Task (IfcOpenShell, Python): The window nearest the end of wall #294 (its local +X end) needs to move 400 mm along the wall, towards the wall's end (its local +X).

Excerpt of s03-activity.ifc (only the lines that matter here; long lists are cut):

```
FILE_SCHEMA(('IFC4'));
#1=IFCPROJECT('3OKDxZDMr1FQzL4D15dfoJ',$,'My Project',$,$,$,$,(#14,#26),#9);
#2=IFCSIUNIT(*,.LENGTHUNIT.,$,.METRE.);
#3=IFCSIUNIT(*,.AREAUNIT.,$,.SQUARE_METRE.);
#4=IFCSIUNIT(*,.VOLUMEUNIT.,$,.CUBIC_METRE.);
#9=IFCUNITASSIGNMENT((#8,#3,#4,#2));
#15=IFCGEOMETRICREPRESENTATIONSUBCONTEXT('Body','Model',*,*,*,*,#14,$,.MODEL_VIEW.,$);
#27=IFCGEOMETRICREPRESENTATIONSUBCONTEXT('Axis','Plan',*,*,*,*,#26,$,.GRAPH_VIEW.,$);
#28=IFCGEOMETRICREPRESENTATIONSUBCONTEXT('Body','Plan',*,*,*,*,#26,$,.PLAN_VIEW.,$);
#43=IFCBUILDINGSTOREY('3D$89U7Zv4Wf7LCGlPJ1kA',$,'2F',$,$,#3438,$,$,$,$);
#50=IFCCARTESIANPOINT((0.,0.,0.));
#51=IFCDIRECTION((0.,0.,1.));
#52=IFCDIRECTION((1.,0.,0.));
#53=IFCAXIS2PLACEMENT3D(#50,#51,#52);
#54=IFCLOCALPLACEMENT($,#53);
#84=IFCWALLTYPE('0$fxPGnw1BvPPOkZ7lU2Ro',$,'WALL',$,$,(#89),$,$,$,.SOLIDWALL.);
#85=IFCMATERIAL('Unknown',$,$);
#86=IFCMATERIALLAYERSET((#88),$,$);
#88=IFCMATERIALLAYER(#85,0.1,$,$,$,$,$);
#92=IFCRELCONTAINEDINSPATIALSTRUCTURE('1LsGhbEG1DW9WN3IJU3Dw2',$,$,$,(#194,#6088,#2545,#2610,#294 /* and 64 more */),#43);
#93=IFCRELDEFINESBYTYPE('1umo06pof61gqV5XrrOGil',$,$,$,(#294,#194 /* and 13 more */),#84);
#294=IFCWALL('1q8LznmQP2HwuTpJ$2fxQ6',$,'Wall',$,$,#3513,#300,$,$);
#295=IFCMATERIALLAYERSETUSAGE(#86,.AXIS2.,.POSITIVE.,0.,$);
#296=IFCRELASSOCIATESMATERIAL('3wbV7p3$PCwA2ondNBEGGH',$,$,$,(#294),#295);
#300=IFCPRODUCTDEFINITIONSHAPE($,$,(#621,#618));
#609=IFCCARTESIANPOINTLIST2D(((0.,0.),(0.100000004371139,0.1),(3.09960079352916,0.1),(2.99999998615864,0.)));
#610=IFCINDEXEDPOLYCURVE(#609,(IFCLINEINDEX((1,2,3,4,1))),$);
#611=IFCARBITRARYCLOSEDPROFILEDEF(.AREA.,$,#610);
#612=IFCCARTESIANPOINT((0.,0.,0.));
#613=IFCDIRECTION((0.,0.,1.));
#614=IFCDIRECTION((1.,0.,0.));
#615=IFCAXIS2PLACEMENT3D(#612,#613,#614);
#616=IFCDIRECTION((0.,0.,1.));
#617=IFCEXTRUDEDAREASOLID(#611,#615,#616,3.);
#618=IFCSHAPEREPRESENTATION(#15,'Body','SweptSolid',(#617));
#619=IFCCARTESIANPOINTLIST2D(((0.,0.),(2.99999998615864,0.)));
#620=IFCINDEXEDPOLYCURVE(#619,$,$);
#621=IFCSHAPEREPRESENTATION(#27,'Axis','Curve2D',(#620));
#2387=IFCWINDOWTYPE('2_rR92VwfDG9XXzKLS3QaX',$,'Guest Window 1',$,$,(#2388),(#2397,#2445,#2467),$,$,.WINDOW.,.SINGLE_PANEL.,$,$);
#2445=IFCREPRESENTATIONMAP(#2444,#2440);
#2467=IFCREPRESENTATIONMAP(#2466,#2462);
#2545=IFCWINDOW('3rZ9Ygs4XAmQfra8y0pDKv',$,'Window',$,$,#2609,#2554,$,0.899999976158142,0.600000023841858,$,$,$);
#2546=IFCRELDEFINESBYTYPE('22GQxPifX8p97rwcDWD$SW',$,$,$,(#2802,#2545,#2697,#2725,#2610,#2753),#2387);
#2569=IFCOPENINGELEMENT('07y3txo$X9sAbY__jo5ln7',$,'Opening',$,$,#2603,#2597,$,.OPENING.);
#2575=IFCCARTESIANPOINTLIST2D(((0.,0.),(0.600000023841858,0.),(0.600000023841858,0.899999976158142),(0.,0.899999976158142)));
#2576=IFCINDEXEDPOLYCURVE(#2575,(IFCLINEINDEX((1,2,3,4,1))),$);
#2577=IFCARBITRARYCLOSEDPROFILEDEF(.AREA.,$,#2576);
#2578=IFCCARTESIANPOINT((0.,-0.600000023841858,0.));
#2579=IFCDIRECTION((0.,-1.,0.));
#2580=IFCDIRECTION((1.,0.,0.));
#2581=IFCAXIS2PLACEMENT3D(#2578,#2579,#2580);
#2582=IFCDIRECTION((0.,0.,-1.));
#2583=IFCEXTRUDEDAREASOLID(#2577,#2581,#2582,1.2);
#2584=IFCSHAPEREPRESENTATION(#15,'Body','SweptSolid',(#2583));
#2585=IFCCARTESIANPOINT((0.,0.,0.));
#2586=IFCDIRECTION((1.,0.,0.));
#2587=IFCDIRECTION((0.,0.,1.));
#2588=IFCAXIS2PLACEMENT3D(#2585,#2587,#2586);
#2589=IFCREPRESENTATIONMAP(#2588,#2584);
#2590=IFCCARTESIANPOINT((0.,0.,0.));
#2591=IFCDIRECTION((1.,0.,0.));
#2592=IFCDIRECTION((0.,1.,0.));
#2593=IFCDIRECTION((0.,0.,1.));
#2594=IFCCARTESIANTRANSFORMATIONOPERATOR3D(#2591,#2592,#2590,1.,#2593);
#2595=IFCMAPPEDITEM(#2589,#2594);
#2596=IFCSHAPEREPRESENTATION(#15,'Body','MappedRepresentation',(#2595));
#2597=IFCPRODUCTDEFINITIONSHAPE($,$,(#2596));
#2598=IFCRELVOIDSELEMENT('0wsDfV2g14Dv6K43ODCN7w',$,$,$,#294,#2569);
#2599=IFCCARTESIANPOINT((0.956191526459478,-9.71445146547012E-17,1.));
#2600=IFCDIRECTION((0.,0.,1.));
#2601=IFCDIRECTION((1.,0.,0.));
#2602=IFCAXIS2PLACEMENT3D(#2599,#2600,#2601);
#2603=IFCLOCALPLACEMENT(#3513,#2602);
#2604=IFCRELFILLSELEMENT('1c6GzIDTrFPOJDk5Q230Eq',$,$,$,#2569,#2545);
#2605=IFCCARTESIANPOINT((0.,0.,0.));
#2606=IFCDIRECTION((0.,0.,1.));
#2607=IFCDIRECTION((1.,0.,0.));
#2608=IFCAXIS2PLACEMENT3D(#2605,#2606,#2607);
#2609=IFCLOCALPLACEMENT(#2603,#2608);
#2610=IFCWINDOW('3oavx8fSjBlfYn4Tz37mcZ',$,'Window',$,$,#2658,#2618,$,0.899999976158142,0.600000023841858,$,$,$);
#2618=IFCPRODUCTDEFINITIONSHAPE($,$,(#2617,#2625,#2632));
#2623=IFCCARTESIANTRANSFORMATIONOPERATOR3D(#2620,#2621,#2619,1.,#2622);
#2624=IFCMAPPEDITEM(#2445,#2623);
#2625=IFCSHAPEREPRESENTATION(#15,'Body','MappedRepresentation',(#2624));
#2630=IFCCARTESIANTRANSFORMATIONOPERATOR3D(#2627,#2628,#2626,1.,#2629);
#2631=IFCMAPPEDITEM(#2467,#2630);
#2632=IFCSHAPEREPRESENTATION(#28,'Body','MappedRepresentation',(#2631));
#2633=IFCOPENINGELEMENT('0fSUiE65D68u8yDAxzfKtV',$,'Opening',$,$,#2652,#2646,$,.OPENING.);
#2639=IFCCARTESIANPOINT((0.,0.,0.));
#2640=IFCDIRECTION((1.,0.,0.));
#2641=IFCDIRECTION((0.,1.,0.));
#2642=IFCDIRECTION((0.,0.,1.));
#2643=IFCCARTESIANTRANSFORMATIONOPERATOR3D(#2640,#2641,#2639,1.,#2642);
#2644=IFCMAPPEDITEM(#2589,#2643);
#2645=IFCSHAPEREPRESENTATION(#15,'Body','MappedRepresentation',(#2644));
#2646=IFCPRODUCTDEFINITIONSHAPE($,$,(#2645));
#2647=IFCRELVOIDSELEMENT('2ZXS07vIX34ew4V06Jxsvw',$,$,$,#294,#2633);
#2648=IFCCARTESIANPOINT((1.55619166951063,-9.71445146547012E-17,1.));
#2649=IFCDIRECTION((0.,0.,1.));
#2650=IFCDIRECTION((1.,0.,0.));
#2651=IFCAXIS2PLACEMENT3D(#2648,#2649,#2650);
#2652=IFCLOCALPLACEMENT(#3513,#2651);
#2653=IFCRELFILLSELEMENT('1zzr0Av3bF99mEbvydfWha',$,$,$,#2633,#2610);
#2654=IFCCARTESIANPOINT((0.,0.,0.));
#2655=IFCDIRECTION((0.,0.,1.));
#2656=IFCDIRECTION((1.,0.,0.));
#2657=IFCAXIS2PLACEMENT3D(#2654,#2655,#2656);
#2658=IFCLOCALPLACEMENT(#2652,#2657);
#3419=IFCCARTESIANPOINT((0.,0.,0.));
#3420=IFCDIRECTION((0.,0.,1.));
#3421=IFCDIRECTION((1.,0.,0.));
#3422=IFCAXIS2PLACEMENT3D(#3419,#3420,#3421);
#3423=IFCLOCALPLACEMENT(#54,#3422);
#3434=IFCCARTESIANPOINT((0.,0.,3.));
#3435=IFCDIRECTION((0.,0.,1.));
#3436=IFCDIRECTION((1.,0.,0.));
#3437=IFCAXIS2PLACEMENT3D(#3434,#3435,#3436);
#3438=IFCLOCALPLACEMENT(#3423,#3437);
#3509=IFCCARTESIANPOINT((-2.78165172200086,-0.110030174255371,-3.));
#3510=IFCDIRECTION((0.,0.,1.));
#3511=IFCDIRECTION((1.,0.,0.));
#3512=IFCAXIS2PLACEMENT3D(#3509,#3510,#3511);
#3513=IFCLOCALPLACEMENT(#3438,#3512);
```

```python
import ifcopenshell
import ifcopenshell.api.geometry
import ifcopenshell.util.placement
import ifcopenshell.util.unit

model = ifcopenshell.open("s03-activity.ifc")
unit_scale = ifcopenshell.util.unit.calculate_unit_scale(model)

window = model.by_guid("3oavx8fSjBlfYn4Tz37mcZ")
opening = window.FillsVoids[0].RelatingOpeningElement
wall = opening.VoidsElements[0].RelatingBuildingElement

wall_matrix = ifcopenshell.util.placement.get_local_placement(wall.ObjectPlacement)
shift = wall_matrix[:3, 0] * 0.4 / unit_scale
before = ifcopenshell.util.placement.get_local_placement(window.ObjectPlacement)[:3, 3].copy()

# The window is placed relative to its opening, so it follows when the opening moves.
matrix = ifcopenshell.util.placement.get_local_placement(opening.ObjectPlacement)
matrix[:3, 3] += shift
ifcopenshell.api.geometry.edit_object_placement(
    model, product=opening, matrix=matrix, is_si=False, should_transform_children=True
)

after = ifcopenshell.util.placement.get_local_placement(window.ObjectPlacement)[:3, 3]
print("window moved by", (after - before).round(3) + 0.0)

model.write("s03-activity_v2.ifc")
```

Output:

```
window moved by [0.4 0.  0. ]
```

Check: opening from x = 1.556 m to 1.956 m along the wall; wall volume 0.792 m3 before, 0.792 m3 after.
